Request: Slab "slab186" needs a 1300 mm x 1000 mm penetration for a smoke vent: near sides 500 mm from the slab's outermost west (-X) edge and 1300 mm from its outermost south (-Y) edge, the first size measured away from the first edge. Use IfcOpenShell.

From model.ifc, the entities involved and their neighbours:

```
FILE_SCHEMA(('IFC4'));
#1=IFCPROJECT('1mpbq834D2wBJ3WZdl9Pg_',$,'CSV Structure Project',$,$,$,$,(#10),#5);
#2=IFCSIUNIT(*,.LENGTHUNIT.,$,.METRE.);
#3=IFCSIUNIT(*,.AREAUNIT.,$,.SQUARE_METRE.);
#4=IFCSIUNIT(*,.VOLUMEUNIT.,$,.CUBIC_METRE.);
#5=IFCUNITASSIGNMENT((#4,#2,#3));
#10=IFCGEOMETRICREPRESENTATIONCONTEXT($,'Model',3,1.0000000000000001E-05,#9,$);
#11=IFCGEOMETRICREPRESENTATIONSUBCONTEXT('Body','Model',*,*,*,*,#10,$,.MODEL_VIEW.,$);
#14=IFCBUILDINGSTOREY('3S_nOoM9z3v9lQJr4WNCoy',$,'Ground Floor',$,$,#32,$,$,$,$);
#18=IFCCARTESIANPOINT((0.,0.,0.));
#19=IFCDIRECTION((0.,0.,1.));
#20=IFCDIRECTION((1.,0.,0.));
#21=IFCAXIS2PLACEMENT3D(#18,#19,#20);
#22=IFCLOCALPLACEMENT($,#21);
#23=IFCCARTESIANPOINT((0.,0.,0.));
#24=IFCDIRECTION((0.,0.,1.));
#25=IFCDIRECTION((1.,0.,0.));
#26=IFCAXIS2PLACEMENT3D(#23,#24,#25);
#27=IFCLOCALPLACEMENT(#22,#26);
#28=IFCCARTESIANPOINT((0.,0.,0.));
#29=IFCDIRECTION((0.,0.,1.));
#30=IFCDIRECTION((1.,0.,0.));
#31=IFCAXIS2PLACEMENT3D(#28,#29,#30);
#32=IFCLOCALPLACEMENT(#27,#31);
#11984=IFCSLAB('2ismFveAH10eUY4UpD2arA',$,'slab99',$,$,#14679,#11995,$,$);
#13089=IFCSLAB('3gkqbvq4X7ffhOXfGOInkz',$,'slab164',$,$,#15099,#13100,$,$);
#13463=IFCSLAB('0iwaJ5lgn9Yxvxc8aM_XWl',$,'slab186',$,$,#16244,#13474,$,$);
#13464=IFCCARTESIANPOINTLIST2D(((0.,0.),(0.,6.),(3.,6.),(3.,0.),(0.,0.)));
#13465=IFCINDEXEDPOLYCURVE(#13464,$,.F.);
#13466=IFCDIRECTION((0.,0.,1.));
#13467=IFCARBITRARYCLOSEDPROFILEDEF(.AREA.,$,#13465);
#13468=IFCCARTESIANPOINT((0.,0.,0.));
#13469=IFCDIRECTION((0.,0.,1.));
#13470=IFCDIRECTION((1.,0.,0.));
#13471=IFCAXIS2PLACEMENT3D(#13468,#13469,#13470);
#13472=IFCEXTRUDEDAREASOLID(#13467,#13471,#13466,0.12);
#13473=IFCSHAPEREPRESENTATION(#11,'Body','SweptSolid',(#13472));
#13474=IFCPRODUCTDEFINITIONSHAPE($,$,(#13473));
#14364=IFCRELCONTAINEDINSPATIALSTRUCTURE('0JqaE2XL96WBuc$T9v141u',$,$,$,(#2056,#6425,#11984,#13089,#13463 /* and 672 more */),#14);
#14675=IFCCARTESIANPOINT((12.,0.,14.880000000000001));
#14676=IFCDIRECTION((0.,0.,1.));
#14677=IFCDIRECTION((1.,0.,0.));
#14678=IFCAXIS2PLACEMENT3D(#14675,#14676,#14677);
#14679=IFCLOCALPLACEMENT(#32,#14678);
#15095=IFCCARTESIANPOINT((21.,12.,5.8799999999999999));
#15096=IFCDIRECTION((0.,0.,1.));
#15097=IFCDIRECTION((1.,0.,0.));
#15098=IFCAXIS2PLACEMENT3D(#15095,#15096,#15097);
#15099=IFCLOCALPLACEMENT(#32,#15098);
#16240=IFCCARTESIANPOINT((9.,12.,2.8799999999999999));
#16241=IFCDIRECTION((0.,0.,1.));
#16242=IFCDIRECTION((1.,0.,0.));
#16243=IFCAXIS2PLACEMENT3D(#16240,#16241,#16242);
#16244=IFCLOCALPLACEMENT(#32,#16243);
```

```python
import numpy as np
import ifcopenshell
import ifcopenshell.api.feature
import ifcopenshell.api.geometry
import ifcopenshell.api.root
import ifcopenshell.geom
import ifcopenshell.util.placement
import ifcopenshell.util.representation
import ifcopenshell.util.shape
import ifcopenshell.util.unit

model = ifcopenshell.open("model.ifc")
unit_scale = ifcopenshell.util.unit.calculate_unit_scale(model)
settings = ifcopenshell.geom.settings()


def volume(element):
    """Net volume in cubic metres, openings subtracted."""
    shape = ifcopenshell.geom.create_shape(settings, element)
    return ifcopenshell.util.shape.get_volume(shape.geometry)


slab = model.by_guid("0iwaJ5lgn9Yxvxc8aM_XWl")
before = volume(slab)

# Extent in the slab's own axes, in metres. The edges named are its -X and -Y sides.
slab_shape = ifcopenshell.geom.create_shape(settings, slab)
vertices = ifcopenshell.util.shape.get_vertices(slab_shape.geometry)
x_min, y_min, bottom = vertices.min(axis=0)
top = vertices[:, 2].max()

opening = ifcopenshell.api.root.create_entity(model, ifc_class="IfcOpeningElement", name="Smoke vent opening", predefined_type="OPENING")
context = ifcopenshell.util.representation.get_context(model, "Model", "Body", "MODEL_VIEW")
width, depth = 1.3, 1
outline = [(0.0, 0.0), (width, 0.0), (width, depth), (0.0, depth), (0.0, 0.0)]
# Overshoot both faces by 50 mm so the cut is clean.
shape = ifcopenshell.api.geometry.add_slab_representation(
    model, context=context, depth=top - bottom + 0.1, polyline=outline
)
ifcopenshell.api.geometry.assign_representation(model, product=opening, representation=shape)

matrix = ifcopenshell.util.placement.get_local_placement(slab.ObjectPlacement)
matrix[:, 3] = matrix @ np.append(np.array([x_min + 0.5, y_min + 1.3, bottom - 0.05]) / unit_scale, 1.0)
ifcopenshell.api.geometry.edit_object_placement(model, product=opening, matrix=matrix, is_si=False)
ifcopenshell.api.feature.add_feature(model, feature=opening, element=slab)

after = volume(slab)

print(f"slab volume {before:.3f} -> {after:.3f} m3")

model.write("model-out.ifc")
```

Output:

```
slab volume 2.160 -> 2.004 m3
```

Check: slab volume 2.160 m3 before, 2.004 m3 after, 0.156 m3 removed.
